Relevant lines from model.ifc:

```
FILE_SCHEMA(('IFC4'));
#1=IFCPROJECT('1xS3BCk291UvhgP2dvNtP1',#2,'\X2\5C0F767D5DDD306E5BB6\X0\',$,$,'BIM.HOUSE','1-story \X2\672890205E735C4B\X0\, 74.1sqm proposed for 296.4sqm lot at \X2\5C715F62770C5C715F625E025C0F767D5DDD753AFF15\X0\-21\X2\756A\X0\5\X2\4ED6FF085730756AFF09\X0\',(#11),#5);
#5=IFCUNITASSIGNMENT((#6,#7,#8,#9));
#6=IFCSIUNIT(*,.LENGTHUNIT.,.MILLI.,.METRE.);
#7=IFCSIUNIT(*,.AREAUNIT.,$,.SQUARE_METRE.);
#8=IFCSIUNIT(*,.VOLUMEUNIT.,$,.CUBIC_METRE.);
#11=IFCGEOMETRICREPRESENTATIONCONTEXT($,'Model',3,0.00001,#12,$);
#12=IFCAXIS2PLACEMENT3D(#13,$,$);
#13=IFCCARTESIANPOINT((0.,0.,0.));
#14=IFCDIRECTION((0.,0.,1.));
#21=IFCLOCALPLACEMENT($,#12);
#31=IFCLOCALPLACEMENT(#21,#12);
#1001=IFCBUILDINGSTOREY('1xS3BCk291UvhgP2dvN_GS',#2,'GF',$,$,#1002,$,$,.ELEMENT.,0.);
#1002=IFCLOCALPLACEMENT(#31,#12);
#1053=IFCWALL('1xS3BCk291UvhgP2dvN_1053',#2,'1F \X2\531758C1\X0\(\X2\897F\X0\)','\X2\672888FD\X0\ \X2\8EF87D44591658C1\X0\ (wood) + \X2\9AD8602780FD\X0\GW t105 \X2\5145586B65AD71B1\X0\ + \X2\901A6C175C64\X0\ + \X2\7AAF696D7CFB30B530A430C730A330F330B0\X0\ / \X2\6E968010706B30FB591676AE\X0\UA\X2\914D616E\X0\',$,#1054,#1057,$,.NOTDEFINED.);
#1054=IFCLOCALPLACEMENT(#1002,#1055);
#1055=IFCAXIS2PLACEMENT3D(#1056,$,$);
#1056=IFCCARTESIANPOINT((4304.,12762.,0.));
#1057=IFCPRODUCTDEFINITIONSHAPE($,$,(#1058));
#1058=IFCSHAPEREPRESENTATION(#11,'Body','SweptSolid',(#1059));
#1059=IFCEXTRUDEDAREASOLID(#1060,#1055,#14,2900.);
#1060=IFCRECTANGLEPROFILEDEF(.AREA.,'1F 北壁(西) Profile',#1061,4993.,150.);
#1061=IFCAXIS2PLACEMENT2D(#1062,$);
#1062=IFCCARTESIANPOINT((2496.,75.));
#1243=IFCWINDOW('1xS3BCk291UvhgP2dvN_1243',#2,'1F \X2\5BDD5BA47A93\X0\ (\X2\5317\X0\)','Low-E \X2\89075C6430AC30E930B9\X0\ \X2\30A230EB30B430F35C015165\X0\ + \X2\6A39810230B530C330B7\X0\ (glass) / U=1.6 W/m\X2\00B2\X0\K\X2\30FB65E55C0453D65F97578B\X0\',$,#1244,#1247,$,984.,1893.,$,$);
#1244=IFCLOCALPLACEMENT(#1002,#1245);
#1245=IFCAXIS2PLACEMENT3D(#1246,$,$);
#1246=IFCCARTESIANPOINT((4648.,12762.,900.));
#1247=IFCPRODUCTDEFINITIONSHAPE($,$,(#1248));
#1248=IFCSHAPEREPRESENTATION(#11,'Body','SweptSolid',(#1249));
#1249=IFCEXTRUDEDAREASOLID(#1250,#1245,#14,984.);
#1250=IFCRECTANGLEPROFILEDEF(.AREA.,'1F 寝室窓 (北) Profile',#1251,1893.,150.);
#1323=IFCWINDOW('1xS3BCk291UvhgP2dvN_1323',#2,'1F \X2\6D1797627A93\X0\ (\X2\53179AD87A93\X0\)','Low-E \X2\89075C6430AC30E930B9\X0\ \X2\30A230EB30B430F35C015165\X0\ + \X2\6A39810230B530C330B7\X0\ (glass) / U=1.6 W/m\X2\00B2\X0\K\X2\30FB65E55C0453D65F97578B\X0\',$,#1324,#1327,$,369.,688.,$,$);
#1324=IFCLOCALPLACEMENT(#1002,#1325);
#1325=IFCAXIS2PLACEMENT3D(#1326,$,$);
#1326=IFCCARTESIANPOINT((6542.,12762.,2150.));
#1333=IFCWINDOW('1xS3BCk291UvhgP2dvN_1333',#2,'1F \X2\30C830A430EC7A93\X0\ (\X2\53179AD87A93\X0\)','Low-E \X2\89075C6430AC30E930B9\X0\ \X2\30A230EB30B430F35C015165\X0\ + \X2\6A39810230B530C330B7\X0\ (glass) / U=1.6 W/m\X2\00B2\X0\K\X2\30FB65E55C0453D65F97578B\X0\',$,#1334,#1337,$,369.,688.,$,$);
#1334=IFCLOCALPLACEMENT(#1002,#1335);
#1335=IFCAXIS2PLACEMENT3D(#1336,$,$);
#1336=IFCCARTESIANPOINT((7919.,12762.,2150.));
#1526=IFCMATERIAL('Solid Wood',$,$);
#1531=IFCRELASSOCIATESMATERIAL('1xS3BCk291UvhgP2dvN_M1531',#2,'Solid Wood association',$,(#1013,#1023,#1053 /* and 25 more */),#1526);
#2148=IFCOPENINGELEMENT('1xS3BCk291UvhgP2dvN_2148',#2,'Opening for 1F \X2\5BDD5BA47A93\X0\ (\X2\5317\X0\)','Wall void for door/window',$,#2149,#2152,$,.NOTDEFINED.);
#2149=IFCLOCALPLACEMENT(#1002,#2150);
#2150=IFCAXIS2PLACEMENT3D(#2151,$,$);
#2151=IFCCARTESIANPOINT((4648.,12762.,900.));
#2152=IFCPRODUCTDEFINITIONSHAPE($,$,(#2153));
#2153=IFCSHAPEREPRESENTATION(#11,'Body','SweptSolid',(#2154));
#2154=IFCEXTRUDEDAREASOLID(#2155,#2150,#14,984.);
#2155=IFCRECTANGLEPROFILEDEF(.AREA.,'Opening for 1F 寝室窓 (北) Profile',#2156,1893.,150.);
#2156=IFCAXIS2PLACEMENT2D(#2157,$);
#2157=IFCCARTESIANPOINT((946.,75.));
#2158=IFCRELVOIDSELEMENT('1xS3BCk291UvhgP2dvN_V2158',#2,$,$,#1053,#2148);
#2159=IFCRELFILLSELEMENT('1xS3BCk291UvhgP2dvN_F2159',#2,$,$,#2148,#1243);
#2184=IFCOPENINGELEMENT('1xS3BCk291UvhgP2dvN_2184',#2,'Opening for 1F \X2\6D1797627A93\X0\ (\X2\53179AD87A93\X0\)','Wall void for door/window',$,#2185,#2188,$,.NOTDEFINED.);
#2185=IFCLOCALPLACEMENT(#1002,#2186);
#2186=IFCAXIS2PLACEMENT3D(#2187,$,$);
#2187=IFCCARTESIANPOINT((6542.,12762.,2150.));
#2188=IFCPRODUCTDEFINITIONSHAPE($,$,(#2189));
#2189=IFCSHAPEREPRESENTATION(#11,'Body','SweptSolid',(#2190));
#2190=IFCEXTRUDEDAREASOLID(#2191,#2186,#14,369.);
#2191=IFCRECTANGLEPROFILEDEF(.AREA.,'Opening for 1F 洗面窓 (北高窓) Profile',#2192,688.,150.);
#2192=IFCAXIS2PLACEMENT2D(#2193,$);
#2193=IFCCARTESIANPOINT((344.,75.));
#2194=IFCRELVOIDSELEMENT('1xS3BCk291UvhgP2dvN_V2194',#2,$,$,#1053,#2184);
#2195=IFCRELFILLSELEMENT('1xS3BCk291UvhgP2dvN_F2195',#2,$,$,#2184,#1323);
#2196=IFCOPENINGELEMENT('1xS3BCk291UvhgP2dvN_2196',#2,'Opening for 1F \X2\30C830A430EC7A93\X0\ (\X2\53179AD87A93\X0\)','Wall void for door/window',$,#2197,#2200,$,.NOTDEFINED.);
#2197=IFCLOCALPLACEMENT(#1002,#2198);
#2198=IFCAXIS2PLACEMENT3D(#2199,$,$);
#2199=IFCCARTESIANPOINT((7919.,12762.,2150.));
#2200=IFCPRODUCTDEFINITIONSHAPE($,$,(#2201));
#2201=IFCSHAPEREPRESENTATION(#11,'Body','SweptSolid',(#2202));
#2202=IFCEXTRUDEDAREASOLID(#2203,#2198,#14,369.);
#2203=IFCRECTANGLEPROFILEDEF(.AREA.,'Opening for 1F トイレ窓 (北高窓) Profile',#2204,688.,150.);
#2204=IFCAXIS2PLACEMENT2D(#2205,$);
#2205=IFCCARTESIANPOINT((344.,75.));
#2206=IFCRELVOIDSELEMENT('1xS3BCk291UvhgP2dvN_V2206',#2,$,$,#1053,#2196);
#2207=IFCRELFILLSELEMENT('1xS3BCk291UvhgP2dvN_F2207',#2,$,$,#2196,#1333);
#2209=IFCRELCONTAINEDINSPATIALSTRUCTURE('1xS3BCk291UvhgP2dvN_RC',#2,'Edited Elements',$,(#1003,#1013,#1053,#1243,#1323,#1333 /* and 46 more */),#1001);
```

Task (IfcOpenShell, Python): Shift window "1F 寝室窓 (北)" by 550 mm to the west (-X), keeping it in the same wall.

```python
import ifcopenshell
import ifcopenshell.api.geometry
import ifcopenshell.util.placement
import ifcopenshell.util.unit

model = ifcopenshell.open("model.ifc")
unit_scale = ifcopenshell.util.unit.calculate_unit_scale(model)

window = model.by_guid("1xS3BCk291UvhgP2dvN_1243")
opening = window.FillsVoids[0].RelatingOpeningElement
wall = opening.VoidsElements[0].RelatingBuildingElement

wall_matrix = ifcopenshell.util.placement.get_local_placement(wall.ObjectPlacement)
shift = wall_matrix[:3, 0] * -0.55 / unit_scale
before = ifcopenshell.util.placement.get_local_placement(window.ObjectPlacement)[:3, 3].copy()

# The window is not placed relative to its opening, so move both.
for product in (opening, window):
    matrix = ifcopenshell.util.placement.get_local_placement(product.ObjectPlacement)
    matrix[:3, 3] += shift
    ifcopenshell.api.geometry.edit_object_placement(model, product=product, matrix=matrix, is_si=False)

after = ifcopenshell.util.placement.get_local_placement(window.ObjectPlacement)[:3, 3]
print("window moved by", (after - before).round(3) + 0.0)

model.write("model_edited.ifc")
```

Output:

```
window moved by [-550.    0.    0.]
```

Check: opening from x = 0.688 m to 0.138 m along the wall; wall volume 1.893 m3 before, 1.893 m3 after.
